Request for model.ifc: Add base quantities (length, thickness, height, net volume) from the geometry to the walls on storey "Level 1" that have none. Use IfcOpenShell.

First a look at what the model holds.

```python
import ifcopenshell
import ifcopenshell.util.element
import ifcopenshell.util.unit

model = ifcopenshell.open("model.ifc")
print(model.schema)
for unit_type in ("LENGTHUNIT", "AREAUNIT", "VOLUMEUNIT"):
    print(unit_type, ifcopenshell.util.unit.calculate_unit_scale(model, unit_type))
storey = next(s for s in model.by_type("IfcBuildingStorey") if s.Name == "Level 1")
walls = [e for e in ifcopenshell.util.element.get_decomposition(storey) if e.is_a("IfcWall")]
for e in sorted(walls, key=lambda e: e.id()):
    print(e.id(), e.is_a(), e.Name, list(ifcopenshell.util.element.get_psets(e, qtos_only=True)), sep=" | ")
```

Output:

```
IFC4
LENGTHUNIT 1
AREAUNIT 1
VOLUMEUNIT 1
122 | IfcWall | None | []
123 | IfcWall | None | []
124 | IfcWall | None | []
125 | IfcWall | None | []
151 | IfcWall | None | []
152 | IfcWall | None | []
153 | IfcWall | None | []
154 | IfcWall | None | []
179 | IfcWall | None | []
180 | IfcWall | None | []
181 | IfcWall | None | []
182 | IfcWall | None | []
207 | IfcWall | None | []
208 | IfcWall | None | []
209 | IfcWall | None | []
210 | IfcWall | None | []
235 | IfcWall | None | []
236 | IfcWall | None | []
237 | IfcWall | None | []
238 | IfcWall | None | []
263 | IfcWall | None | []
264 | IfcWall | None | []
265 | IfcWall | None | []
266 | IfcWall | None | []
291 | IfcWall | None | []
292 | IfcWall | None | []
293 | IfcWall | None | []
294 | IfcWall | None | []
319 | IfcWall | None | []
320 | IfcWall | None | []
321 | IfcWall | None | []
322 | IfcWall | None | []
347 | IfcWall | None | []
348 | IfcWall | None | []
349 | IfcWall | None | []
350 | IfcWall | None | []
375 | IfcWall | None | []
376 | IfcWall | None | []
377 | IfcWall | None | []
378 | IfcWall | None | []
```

```python
import ifcopenshell
import ifcopenshell.api.pset
import ifcopenshell.geom
import ifcopenshell.util.element
import ifcopenshell.util.shape
import ifcopenshell.util.unit

model = ifcopenshell.open("model.ifc")
unit_scale = ifcopenshell.util.unit.calculate_unit_scale(model)
volume_scale = ifcopenshell.util.unit.calculate_unit_scale(model, "VOLUMEUNIT")
settings = ifcopenshell.geom.settings()

storey = next(s for s in model.by_type("IfcBuildingStorey") if s.Name == "Level 1")
walls = [e for e in ifcopenshell.util.element.get_decomposition(storey) if e.is_a("IfcWall")]

for e in sorted(walls, key=lambda e: e.id()):
    if ifcopenshell.util.element.get_psets(e, qtos_only=True, should_inherit=False):
        continue
    # Geometry comes back in metres, in the element's own axes.
    shape = ifcopenshell.geom.create_shape(settings, e)
    values = {
        "Length": ifcopenshell.util.shape.get_x(shape.geometry) / unit_scale,
        "Width": ifcopenshell.util.shape.get_y(shape.geometry) / unit_scale,
        "Height": ifcopenshell.util.shape.get_z(shape.geometry) / unit_scale,
        "NetVolume": ifcopenshell.util.shape.get_volume(shape.geometry) / volume_scale,
    }
    qto = ifcopenshell.api.pset.add_qto(model, product=e, name="Qto_WallBaseQuantities")
    ifcopenshell.api.pset.edit_qto(model, qto=qto, properties=values)
    print(e.id(), {k: round(v, 3) for k, v in values.items()})

model.write("model_v2.ifc")
```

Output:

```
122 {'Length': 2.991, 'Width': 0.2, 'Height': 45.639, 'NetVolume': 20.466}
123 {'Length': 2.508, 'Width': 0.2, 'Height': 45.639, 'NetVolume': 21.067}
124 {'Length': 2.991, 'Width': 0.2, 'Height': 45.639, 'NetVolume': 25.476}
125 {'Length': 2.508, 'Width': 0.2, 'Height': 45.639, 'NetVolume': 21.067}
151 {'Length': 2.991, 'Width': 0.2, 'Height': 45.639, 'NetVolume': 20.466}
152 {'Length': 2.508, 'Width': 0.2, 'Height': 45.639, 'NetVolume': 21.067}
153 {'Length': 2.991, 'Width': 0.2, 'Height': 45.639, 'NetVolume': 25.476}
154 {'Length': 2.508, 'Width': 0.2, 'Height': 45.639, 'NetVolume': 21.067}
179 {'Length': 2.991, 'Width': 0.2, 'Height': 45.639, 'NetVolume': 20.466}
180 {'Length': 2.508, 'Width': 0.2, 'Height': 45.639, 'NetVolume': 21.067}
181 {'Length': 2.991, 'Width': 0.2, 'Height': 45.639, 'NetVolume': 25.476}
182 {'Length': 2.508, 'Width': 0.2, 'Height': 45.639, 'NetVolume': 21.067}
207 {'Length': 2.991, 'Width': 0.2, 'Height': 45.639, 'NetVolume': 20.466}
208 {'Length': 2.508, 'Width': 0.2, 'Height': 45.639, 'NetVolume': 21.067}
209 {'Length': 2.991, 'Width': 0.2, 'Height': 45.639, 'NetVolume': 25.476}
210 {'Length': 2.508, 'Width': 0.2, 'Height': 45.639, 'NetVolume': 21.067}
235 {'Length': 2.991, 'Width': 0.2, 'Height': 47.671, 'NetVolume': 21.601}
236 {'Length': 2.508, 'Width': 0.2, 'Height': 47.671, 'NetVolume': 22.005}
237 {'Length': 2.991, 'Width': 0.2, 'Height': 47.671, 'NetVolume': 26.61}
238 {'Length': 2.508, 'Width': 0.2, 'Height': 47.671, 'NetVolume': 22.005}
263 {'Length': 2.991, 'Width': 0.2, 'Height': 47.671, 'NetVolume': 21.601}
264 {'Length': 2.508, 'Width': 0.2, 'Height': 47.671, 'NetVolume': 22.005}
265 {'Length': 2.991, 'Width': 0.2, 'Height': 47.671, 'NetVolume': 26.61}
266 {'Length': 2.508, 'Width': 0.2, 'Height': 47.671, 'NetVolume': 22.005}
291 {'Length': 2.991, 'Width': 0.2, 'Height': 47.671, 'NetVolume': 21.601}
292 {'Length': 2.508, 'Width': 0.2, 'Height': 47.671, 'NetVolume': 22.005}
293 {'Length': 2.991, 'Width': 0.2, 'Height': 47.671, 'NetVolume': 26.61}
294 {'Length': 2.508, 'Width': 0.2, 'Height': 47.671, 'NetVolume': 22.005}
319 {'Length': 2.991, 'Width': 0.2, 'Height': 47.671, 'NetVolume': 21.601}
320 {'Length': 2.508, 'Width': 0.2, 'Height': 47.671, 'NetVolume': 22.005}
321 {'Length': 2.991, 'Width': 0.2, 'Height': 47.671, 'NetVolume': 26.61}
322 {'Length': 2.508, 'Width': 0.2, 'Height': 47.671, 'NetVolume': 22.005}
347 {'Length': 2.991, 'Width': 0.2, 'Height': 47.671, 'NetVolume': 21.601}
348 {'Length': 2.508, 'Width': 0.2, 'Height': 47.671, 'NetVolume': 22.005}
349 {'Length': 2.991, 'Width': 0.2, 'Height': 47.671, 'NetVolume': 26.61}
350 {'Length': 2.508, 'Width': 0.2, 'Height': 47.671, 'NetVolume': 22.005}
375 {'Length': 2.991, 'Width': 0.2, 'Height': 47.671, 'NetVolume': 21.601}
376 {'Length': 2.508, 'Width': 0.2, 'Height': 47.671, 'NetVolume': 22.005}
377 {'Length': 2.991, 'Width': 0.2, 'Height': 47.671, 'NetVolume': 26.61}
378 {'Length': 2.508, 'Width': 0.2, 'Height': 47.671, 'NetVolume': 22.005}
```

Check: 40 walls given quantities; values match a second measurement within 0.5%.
